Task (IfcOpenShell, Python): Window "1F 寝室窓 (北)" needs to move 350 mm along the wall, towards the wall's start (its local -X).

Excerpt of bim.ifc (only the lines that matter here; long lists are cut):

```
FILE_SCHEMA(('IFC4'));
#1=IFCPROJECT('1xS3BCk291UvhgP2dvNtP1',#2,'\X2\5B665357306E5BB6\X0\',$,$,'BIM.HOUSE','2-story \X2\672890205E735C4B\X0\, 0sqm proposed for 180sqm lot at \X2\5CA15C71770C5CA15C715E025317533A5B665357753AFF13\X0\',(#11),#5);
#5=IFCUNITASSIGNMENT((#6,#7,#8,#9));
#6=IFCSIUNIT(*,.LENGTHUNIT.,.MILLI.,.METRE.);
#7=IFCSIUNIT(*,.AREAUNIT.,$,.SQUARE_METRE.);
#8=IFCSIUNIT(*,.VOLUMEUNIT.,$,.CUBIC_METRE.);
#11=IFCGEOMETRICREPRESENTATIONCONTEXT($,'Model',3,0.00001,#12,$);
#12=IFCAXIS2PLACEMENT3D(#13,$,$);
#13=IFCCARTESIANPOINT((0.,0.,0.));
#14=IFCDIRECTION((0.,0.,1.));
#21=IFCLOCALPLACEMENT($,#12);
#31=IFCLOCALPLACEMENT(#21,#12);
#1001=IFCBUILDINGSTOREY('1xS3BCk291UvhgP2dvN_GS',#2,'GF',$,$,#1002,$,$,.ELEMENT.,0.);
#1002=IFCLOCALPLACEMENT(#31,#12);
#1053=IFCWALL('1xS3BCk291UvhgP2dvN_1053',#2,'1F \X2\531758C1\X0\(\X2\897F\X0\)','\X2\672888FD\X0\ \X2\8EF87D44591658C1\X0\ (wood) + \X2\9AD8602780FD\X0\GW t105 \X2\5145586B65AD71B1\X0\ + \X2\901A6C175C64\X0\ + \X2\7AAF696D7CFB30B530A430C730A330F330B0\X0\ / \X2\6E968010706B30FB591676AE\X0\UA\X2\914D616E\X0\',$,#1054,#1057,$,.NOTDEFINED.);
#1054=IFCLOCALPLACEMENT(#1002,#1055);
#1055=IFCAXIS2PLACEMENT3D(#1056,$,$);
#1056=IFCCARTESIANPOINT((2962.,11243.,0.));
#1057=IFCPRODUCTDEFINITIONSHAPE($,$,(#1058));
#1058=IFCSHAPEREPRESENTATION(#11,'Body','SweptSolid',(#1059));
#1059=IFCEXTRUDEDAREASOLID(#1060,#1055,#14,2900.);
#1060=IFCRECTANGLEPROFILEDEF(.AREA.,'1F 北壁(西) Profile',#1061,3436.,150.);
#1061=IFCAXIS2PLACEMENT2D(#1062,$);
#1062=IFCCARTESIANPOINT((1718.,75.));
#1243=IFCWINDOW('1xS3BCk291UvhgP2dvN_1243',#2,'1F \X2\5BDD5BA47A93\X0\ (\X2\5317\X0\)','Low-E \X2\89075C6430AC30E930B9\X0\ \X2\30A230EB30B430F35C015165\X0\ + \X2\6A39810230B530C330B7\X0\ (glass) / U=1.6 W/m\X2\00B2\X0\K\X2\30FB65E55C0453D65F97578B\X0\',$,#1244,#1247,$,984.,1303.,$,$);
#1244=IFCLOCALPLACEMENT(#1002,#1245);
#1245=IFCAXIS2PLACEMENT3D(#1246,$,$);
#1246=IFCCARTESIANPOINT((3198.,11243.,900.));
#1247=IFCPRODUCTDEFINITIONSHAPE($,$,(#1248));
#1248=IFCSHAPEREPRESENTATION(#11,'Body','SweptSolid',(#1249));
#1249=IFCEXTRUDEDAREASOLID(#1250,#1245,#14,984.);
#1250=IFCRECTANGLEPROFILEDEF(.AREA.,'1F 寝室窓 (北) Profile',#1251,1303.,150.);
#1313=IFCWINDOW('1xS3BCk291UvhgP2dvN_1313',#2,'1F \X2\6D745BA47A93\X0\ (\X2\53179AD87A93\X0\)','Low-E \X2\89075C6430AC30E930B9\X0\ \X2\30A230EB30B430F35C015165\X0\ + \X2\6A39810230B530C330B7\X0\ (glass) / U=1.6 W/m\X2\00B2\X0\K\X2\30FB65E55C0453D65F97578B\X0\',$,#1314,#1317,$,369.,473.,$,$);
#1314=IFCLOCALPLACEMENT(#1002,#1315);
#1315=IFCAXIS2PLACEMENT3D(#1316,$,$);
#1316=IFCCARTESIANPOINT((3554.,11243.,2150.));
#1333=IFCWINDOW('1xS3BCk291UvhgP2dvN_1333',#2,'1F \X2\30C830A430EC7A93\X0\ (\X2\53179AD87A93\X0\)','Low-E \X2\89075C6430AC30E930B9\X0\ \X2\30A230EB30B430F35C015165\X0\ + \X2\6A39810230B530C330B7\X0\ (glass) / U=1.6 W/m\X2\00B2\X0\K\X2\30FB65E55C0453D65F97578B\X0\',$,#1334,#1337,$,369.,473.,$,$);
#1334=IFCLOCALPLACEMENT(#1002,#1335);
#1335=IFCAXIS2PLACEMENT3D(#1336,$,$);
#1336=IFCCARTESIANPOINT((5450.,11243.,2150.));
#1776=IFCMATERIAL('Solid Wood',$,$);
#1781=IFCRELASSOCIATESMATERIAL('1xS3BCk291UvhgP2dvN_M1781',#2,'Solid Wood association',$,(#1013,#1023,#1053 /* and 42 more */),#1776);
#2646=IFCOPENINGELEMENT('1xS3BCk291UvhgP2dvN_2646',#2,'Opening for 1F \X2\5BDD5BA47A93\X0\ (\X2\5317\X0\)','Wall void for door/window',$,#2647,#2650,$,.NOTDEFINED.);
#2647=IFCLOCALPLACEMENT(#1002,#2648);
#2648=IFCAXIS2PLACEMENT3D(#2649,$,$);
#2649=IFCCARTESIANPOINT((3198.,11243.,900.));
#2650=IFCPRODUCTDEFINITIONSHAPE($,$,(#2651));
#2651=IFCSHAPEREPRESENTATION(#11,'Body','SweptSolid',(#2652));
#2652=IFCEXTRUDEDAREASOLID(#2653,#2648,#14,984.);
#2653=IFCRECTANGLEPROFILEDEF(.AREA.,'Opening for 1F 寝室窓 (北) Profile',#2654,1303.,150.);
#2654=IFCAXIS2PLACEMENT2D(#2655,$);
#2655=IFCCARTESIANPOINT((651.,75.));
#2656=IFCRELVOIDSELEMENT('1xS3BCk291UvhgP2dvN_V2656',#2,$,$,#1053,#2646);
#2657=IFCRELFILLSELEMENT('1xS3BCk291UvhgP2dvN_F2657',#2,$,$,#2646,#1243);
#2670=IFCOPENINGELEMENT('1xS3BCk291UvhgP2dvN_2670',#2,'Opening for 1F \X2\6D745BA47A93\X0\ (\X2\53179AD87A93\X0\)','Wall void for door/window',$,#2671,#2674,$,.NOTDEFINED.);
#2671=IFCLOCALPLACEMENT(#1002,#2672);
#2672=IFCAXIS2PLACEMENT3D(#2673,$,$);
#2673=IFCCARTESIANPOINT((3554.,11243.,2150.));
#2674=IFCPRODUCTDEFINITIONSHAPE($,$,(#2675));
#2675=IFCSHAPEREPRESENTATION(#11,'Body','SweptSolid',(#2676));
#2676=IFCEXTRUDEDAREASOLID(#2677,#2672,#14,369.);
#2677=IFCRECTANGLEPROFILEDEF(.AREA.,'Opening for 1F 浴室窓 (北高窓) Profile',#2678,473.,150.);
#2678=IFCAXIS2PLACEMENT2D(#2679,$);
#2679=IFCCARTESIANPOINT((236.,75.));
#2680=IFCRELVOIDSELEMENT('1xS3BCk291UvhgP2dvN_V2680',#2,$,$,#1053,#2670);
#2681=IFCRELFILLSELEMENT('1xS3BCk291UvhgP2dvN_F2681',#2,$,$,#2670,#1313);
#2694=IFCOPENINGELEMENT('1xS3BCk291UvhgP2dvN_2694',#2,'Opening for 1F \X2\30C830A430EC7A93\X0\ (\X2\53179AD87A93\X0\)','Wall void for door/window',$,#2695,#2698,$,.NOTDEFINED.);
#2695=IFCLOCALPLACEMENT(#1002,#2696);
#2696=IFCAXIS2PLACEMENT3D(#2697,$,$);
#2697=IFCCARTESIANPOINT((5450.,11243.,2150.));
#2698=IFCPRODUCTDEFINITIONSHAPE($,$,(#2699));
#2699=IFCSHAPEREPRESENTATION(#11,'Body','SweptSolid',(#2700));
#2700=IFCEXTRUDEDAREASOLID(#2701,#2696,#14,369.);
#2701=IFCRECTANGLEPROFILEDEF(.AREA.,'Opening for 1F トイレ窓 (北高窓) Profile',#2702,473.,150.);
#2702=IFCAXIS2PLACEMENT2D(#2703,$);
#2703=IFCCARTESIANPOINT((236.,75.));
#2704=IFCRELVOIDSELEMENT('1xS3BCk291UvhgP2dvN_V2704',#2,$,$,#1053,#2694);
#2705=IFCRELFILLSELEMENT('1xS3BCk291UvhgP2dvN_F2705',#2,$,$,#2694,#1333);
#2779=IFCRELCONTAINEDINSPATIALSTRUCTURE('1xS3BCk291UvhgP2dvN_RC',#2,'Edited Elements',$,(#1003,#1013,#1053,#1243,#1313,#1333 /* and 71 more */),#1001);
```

```python
import ifcopenshell
import ifcopenshell.api.geometry
import ifcopenshell.util.placement

model = ifcopenshell.open("bim.ifc")

window = model.by_id(1243)
opening = window.FillsVoids[0].RelatingOpeningElement
wall = opening.VoidsElements[0].RelatingBuildingElement

wall_matrix = ifcopenshell.util.placement.get_local_placement(wall.ObjectPlacement)
shift = wall_matrix[:3, 0] * -350.0
before = ifcopenshell.util.placement.get_local_placement(window.ObjectPlacement)[:3, 3].copy()

# The window is not placed relative to its opening, so move both.
for product in (opening, window):
    matrix = ifcopenshell.util.placement.get_local_placement(product.ObjectPlacement)
    matrix[:3, 3] += shift
    ifcopenshell.api.geometry.edit_object_placement(model, product=product, matrix=matrix, is_si=False)

after = ifcopenshell.util.placement.get_local_placement(window.ObjectPlacement)[:3, 3]
print("window moved by", (after - before).round(3) + 0.0)

model.write("bim_v2.ifc")
```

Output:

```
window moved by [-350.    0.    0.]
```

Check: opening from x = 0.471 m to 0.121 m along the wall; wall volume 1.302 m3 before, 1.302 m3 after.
